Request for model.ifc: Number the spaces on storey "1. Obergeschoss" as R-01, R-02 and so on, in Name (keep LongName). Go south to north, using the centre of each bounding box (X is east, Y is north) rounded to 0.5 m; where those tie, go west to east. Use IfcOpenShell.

First a look at what the model holds.

```python
import ifcopenshell
import ifcopenshell.util.element
import ifcopenshell.util.placement

model = ifcopenshell.open("model.ifc")
print(model.schema)
storey = next(s for s in model.by_type("IfcBuildingStorey") if s.Name == "1. Obergeschoss")
spaces = [e for e in ifcopenshell.util.element.get_decomposition(storey) if e.is_a("IfcSpace")]
for e in sorted(spaces, key=lambda e: e.id()):
    origin = ifcopenshell.util.placement.get_local_placement(e.ObjectPlacement)[:3, 3]
    print(e.id(), e.Name, e.LongName, origin.round(2) + 0.0, sep=" | ")
```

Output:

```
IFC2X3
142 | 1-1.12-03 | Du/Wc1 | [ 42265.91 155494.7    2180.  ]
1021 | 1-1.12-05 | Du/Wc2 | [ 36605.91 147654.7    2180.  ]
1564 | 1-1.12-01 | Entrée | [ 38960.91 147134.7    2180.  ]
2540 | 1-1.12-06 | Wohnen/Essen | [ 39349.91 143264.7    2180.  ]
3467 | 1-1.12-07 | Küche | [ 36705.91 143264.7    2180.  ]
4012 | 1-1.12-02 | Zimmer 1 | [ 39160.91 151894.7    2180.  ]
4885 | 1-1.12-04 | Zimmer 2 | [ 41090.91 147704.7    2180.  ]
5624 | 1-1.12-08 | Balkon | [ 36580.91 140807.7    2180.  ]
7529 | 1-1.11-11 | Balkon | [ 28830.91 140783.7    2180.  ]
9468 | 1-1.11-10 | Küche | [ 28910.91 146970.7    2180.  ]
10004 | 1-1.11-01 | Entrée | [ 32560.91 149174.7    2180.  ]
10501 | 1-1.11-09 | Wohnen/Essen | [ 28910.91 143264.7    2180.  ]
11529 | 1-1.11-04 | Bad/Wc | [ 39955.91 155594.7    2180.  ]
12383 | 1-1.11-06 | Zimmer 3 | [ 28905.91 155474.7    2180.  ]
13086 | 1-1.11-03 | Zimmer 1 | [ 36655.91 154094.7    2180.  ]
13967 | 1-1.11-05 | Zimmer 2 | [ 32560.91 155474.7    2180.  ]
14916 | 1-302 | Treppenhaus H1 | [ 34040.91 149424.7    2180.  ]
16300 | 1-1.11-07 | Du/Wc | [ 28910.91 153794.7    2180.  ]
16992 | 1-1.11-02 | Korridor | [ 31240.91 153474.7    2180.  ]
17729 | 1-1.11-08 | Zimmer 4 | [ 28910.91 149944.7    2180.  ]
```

```python
import ifcopenshell
import ifcopenshell.geom
import ifcopenshell.util.element
import ifcopenshell.util.shape

model = ifcopenshell.open("model.ifc")
settings = ifcopenshell.geom.settings()
settings.set("use-world-coords", True)


def centre(element):
    shape = ifcopenshell.geom.create_shape(settings, element)
    return ifcopenshell.util.shape.get_bbox_centroid(shape.geometry)


storey = next(s for s in model.by_type("IfcBuildingStorey") if s.Name == "1. Obergeschoss")
spaces = [e for e in ifcopenshell.util.element.get_decomposition(storey) if e.is_a("IfcSpace")]

# Insertion points can sit at a corner or the storey origin, so sort by the geometry (in metres).
centres = {e: centre(e) for e in spaces}
spaces.sort(key=lambda e: (round(centres[e][1] / 0.5), centres[e][0]))

for i, e in enumerate(spaces, start=1):
    number = f"R-{i:02d}"
    e.Name = number
    print(e.id(), number)

model.write("model-out.ifc")
```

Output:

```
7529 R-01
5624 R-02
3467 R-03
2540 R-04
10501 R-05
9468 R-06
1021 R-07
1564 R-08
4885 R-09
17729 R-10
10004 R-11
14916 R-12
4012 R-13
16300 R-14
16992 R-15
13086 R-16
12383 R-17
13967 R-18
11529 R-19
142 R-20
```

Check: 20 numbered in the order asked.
